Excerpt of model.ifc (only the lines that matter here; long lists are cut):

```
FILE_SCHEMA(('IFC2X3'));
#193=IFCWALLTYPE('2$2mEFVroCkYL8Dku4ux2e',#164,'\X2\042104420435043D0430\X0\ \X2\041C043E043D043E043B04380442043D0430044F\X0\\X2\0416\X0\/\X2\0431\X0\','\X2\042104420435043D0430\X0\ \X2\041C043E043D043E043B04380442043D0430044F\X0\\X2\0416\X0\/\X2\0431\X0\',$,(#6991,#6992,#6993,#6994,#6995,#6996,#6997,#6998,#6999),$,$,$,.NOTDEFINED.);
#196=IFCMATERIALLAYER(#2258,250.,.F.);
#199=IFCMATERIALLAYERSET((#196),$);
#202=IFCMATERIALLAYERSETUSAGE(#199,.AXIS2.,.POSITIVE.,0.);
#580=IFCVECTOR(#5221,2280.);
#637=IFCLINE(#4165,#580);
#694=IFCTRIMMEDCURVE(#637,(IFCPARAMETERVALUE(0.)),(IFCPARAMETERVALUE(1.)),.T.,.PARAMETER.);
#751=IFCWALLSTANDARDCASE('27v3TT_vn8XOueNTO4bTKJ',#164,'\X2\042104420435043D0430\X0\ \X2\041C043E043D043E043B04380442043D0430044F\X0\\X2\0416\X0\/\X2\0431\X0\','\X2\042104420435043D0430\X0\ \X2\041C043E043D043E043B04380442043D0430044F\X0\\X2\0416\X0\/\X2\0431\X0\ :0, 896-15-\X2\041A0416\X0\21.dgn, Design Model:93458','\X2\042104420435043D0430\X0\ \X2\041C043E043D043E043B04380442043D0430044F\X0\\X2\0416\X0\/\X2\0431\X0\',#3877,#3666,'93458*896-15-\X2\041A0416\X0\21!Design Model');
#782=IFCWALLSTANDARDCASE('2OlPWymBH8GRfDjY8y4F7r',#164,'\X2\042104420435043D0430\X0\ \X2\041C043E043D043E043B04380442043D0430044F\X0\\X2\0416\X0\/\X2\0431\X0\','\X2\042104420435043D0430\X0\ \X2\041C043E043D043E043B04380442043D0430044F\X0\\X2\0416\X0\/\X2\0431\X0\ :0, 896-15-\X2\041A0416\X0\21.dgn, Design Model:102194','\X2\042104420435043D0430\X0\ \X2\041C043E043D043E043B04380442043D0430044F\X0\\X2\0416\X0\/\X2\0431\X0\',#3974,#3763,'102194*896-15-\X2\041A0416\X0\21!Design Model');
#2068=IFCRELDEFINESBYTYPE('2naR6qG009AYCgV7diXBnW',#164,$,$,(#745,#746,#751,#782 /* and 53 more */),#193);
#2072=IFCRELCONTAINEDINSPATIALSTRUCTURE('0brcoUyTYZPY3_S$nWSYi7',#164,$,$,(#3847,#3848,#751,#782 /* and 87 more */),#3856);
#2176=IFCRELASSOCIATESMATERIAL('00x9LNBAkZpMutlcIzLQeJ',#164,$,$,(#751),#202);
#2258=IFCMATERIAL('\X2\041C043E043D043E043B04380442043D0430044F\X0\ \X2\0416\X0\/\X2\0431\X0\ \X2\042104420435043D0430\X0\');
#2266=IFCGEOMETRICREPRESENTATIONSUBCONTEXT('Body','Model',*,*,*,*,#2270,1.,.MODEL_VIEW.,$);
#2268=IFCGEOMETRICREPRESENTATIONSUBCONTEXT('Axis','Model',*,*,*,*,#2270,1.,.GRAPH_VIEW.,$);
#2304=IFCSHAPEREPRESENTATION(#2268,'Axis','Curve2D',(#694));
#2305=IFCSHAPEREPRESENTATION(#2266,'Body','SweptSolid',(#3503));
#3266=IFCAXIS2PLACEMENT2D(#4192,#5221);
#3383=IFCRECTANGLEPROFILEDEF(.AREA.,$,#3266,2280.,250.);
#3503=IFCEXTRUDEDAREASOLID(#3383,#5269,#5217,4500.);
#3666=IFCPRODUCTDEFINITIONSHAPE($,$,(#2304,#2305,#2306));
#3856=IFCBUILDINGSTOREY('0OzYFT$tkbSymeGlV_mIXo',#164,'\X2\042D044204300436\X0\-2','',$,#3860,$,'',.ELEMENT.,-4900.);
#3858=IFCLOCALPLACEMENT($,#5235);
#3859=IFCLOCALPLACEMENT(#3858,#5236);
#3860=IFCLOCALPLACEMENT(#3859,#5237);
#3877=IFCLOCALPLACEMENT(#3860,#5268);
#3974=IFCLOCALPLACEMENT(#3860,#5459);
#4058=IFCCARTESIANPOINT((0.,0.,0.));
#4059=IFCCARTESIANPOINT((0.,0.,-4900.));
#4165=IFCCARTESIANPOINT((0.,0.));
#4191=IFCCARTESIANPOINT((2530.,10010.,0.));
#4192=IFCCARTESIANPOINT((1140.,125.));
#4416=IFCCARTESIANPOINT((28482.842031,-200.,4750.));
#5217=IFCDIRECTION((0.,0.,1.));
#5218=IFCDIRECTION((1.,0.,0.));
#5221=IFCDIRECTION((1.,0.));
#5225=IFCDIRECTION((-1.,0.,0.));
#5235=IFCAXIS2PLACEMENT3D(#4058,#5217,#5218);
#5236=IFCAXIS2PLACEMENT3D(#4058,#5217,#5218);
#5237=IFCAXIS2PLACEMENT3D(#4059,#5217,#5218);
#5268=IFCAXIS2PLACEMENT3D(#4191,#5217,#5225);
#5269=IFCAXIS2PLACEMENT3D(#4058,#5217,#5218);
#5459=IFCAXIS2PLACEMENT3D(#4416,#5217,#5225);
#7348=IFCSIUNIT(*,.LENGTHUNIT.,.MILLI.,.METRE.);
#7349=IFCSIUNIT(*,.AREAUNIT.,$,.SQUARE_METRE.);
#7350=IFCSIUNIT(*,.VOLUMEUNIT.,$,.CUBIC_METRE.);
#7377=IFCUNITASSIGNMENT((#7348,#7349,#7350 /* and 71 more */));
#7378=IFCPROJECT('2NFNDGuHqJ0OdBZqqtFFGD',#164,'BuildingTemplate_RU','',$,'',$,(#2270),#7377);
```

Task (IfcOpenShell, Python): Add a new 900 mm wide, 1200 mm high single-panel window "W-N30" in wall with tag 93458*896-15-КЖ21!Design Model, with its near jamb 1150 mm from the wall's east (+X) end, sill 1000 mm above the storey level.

```python
import numpy as np
import ifcopenshell
import ifcopenshell.api.feature
import ifcopenshell.api.geometry
import ifcopenshell.api.root
import ifcopenshell.api.spatial
import ifcopenshell.api.type
import ifcopenshell.geom
import ifcopenshell.util.element
import ifcopenshell.util.placement
import ifcopenshell.util.representation
import ifcopenshell.util.shape
import ifcopenshell.util.unit

model = ifcopenshell.open("model.ifc")
unit_scale = ifcopenshell.util.unit.calculate_unit_scale(model)
settings = ifcopenshell.geom.settings()


def volume(element):
    """Net volume in cubic metres, openings subtracted."""
    shape = ifcopenshell.geom.create_shape(settings, element)
    return ifcopenshell.util.shape.get_volume(shape.geometry)


wall = model.by_guid("27v3TT_vn8XOueNTO4bTKJ")
storey = ifcopenshell.util.element.get_container(wall, ifc_class="IfcBuildingStorey")
context = ifcopenshell.util.representation.get_context(model, "Model", "Body", "MODEL_VIEW")
before = volume(wall)

width, height, from_end, sill = 0.9, 1.2, 1.15, 1  # metres

# The wall runs along its own X axis, and the end named is its -X end.
wall_shape = ifcopenshell.geom.create_shape(settings, wall)
x, y, z = ifcopenshell.util.shape.get_vertices(wall_shape.geometry).T
start = x.min() + from_end
face, thickness = float(y.min()), float(y.max() - y.min())
wall_matrix = ifcopenshell.util.placement.get_local_placement(wall.ObjectPlacement)
level = ifcopenshell.util.placement.get_local_placement(storey.ObjectPlacement)[2, 3]


def in_wall(x, y):
    """Placement at x, y metres in the wall's axes, at sill height."""
    matrix = wall_matrix.copy()
    matrix[:, 3] = wall_matrix @ np.array([x / unit_scale, y / unit_scale, 0.0, 1.0])
    matrix[2, 3] = level + sill / unit_scale
    return matrix


# Opening: a box that overshoots both wall faces by 50 mm.
opening = ifcopenshell.api.root.create_entity(model, ifc_class="IfcOpeningElement")
box = ifcopenshell.api.geometry.add_wall_representation(
    model, context=context, length=width, height=height, thickness=thickness + 0.1
)
ifcopenshell.api.geometry.assign_representation(model, product=opening, representation=box)
ifcopenshell.api.geometry.edit_object_placement(model, product=opening, matrix=in_wall(start, face - 0.05), is_si=False)
ifcopenshell.api.feature.add_feature(model, feature=opening, element=wall)

window = ifcopenshell.api.root.create_entity(model, ifc_class="IfcWindow", name="W-N30")
window.OverallWidth, window.OverallHeight = width / unit_scale, height / unit_scale
body = ifcopenshell.api.geometry.add_window_representation(
    model,
    context=context,
    overall_width=window.OverallWidth,
    overall_height=window.OverallHeight,
    partition_type="SINGLE_PANEL",
)
ifcopenshell.api.geometry.assign_representation(model, product=window, representation=body)
ifcopenshell.api.spatial.assign_container(model, products=[window], relating_structure=storey)
fills = ifcopenshell.api.feature.add_filling(model, opening=opening, element=window)
fills.OwnerHistory = window.OwnerHistory  # required in IFC2X3

# IFC2X3 keeps the operation on the window style.
style = ifcopenshell.api.root.create_entity(model, ifc_class="IfcWindowStyle", name="W-N30")
style.OperationType, style.ConstructionType = "SINGLE_PANEL", "NOTDEFINED"
style.ParameterTakesPrecedence = style.Sizeable = False
ifcopenshell.api.type.assign_type(model, related_objects=[window], relating_type=style)

# Centre the window in the wall's thickness.
ifcopenshell.api.geometry.edit_object_placement(model, product=window, matrix=in_wall(start, face), is_si=False)
window_shape = ifcopenshell.geom.create_shape(settings, window)
depth = ifcopenshell.util.shape.get_vertices(window_shape.geometry)[:, 1]
offset = face + thickness / 2 - (depth.min() + depth.max()) / 2
ifcopenshell.api.geometry.edit_object_placement(model, product=window, matrix=in_wall(start, offset), is_si=False)

after = volume(wall)

print(f"wall volume {before:.3f} -> {after:.3f} m3")

model.write("model_edited.ifc")
```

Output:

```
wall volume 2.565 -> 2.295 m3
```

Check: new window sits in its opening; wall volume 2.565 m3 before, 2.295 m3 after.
